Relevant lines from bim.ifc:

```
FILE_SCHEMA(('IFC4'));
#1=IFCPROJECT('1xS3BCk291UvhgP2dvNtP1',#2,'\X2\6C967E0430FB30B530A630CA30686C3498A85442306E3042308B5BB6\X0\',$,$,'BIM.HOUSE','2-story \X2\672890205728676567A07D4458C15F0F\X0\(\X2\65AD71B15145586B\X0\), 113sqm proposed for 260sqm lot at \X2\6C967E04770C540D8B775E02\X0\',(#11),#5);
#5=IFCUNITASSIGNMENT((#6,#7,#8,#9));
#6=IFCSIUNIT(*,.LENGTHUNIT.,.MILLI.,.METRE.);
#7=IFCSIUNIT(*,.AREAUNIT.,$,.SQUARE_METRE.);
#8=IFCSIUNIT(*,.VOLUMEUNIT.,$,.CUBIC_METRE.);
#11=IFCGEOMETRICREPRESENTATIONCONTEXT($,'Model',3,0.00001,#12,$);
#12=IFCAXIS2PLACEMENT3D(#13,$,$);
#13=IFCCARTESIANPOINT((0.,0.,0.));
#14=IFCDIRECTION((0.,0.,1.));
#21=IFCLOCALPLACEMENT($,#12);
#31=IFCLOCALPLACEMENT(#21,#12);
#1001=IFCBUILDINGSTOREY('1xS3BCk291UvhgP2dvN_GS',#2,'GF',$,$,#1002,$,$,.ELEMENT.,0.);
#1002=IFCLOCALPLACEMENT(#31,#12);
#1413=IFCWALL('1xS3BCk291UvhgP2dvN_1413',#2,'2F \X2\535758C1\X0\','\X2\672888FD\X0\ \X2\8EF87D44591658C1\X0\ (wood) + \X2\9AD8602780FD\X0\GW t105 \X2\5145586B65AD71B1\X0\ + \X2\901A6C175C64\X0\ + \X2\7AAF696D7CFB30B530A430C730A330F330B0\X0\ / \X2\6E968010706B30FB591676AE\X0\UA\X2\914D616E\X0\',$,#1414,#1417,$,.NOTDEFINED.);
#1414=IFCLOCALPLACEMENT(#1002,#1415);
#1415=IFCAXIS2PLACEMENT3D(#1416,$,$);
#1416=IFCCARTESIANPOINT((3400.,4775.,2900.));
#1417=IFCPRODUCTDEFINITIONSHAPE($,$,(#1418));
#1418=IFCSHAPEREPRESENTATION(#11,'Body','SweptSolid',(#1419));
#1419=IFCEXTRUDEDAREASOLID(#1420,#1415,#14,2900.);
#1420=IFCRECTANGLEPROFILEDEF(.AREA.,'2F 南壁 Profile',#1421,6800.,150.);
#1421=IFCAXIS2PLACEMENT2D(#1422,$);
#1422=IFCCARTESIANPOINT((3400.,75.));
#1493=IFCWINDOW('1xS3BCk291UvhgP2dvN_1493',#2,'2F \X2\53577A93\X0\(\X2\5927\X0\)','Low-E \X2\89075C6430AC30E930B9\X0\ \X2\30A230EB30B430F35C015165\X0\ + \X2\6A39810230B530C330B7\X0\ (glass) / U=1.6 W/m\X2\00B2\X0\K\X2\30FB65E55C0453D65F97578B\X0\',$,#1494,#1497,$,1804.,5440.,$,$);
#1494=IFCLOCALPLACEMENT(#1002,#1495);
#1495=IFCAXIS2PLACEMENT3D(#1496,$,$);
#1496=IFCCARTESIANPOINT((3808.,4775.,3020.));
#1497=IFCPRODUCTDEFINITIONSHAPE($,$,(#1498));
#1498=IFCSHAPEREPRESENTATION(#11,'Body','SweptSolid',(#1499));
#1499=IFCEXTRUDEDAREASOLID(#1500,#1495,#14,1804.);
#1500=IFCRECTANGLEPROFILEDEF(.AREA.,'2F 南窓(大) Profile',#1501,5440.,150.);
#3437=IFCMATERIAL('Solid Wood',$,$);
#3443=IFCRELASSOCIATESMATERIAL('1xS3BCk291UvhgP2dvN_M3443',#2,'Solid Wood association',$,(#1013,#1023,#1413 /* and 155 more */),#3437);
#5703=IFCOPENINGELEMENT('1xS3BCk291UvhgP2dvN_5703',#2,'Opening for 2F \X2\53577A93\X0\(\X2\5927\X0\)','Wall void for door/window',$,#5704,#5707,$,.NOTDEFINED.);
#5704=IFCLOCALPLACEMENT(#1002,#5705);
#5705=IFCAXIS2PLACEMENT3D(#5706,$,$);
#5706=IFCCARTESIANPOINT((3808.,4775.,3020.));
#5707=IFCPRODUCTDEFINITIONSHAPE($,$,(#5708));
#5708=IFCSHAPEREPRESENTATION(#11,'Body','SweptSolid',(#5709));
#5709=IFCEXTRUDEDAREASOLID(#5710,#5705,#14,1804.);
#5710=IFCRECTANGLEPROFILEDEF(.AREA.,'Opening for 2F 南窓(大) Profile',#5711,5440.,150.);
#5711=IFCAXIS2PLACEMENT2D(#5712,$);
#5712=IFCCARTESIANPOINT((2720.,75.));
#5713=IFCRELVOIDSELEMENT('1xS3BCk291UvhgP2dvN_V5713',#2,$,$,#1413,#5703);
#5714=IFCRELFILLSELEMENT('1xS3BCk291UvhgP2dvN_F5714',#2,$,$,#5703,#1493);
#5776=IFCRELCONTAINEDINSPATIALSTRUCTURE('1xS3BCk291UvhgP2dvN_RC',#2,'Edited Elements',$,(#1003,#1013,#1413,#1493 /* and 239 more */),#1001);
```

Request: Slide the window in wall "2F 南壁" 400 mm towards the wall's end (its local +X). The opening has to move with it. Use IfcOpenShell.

```python
import ifcopenshell
import ifcopenshell.api.geometry
import ifcopenshell.util.placement

model = ifcopenshell.open("bim.ifc")

window = model.by_id(1493)
opening = window.FillsVoids[0].RelatingOpeningElement
wall = opening.VoidsElements[0].RelatingBuildingElement

wall_matrix = ifcopenshell.util.placement.get_local_placement(wall.ObjectPlacement)
shift = wall_matrix[:3, 0] * 400.0
before = ifcopenshell.util.placement.get_local_placement(window.ObjectPlacement)[:3, 3].copy()

# The window is not placed relative to its opening, so move both.
for product in (opening, window):
    matrix = ifcopenshell.util.placement.get_local_placement(product.ObjectPlacement)
    matrix[:3, 3] += shift
    ifcopenshell.api.geometry.edit_object_placement(model, product=product, matrix=matrix, is_si=False)

after = ifcopenshell.util.placement.get_local_placement(window.ObjectPlacement)[:3, 3]
print("window moved by", (after - before).round(3) + 0.0)

model.write("bim_rev.ifc")
```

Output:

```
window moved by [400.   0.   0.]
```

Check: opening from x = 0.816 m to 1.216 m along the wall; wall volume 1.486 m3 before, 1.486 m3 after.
